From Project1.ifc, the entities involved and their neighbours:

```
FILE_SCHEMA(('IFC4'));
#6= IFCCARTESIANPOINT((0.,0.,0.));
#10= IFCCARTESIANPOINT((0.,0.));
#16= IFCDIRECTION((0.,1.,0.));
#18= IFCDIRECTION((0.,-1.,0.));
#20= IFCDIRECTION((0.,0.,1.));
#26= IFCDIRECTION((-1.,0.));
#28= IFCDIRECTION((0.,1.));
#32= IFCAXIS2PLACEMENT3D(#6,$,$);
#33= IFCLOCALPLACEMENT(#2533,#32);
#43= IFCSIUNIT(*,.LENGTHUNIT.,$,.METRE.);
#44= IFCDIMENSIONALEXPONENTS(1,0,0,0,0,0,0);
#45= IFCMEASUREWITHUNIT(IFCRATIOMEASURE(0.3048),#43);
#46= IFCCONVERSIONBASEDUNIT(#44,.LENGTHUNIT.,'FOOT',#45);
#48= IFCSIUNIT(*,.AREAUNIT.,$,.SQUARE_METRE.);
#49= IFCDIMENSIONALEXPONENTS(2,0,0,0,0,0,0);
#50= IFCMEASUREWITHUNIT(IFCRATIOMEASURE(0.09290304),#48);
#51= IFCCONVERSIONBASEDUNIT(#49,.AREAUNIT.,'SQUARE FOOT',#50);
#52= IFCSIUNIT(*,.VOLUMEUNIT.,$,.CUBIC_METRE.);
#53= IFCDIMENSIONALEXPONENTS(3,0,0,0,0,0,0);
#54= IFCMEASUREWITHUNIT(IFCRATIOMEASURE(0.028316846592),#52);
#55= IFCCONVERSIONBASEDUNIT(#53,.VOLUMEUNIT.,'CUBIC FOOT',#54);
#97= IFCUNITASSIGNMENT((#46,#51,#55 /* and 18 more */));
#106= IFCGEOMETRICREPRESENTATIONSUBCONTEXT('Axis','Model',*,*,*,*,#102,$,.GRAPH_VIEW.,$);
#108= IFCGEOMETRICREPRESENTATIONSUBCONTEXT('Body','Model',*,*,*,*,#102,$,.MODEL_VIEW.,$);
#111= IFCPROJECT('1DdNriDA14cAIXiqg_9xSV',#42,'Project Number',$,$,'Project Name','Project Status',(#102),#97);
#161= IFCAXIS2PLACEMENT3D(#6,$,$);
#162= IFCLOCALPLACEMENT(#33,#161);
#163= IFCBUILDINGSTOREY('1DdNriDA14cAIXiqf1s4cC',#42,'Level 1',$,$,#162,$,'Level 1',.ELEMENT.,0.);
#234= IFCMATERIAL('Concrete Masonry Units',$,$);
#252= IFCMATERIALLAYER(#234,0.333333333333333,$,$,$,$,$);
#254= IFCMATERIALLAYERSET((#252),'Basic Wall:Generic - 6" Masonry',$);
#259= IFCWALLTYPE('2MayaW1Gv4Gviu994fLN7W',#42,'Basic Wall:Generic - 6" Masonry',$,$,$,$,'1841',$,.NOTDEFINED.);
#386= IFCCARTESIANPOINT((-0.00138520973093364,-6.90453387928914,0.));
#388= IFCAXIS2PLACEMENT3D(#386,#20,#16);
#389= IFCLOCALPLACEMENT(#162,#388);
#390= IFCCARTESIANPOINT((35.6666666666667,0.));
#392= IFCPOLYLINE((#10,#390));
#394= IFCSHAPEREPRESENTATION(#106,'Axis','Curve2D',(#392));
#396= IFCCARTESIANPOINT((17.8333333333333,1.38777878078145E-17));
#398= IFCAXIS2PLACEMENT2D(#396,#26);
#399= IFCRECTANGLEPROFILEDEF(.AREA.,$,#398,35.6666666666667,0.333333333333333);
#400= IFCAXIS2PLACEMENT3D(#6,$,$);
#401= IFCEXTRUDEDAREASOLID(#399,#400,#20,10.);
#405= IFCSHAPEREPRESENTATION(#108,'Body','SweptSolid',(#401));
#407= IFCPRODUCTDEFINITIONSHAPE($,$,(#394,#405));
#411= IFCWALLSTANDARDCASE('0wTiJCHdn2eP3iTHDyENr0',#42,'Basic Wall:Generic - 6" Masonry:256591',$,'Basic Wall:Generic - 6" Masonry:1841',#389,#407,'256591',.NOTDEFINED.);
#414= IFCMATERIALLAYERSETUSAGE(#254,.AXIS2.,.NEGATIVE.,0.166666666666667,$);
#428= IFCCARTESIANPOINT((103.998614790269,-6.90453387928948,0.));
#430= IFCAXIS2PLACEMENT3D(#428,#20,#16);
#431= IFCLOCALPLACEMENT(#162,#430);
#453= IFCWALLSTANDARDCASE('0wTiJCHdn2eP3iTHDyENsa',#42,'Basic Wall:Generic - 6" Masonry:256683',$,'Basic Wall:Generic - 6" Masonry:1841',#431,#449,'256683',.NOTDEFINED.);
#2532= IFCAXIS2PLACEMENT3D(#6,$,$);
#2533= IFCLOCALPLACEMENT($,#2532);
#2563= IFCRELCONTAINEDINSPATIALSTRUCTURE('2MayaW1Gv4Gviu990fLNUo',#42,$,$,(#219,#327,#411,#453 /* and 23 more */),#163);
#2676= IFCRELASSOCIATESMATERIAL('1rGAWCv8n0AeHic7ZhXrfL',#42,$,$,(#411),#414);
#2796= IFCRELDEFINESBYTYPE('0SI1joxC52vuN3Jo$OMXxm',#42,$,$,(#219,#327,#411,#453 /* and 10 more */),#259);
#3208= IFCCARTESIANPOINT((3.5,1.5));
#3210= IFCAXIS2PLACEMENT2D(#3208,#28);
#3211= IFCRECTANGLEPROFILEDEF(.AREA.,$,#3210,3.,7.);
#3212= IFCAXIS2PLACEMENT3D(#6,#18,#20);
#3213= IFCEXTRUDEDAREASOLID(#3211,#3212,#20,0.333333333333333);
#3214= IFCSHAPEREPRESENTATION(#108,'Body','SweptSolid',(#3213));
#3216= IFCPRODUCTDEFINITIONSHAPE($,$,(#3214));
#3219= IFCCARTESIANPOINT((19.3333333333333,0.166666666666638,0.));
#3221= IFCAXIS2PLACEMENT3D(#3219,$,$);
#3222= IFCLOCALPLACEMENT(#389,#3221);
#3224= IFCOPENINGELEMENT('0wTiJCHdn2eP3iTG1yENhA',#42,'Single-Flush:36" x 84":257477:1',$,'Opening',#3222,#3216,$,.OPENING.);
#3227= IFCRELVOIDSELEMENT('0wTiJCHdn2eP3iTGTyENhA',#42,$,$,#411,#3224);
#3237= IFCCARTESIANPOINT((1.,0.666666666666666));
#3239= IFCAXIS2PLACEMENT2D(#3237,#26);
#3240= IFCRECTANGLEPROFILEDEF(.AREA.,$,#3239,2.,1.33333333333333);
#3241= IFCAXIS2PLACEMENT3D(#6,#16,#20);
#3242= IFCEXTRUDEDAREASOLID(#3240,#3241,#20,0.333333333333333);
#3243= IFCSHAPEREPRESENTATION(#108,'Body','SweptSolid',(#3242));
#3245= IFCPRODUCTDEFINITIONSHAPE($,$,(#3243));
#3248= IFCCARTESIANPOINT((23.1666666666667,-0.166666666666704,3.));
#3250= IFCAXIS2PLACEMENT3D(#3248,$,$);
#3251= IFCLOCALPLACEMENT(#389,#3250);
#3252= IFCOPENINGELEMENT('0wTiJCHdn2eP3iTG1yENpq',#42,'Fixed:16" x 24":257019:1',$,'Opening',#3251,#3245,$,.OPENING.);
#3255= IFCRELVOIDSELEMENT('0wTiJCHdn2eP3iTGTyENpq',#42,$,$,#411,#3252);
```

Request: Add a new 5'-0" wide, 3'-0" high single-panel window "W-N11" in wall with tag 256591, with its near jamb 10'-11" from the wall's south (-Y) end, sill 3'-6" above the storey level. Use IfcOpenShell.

```python
import numpy as np
import ifcopenshell
import ifcopenshell.api.feature
import ifcopenshell.api.geometry
import ifcopenshell.api.root
import ifcopenshell.api.spatial
import ifcopenshell.geom
import ifcopenshell.util.element
import ifcopenshell.util.placement
import ifcopenshell.util.representation
import ifcopenshell.util.shape
import ifcopenshell.util.unit

model = ifcopenshell.open("Project1.ifc")
unit_scale = ifcopenshell.util.unit.calculate_unit_scale(model)
settings = ifcopenshell.geom.settings()


def volume(element):
    """Net volume in cubic metres, openings subtracted."""
    shape = ifcopenshell.geom.create_shape(settings, element)
    return ifcopenshell.util.shape.get_volume(shape.geometry)


wall = model.by_id(411)
storey = ifcopenshell.util.element.get_container(wall, ifc_class="IfcBuildingStorey")
context = ifcopenshell.util.representation.get_context(model, "Model", "Body", "MODEL_VIEW")
before = volume(wall)

width, height, from_end, sill = 1.524, 0.9144, 3.3274, 1.0668  # metres

# The wall runs along its own X axis, and the end named is its -X end.
wall_shape = ifcopenshell.geom.create_shape(settings, wall)
x, y, z = ifcopenshell.util.shape.get_vertices(wall_shape.geometry).T
start = x.min() + from_end
face, thickness = float(y.min()), float(y.max() - y.min())
wall_matrix = ifcopenshell.util.placement.get_local_placement(wall.ObjectPlacement)
level = ifcopenshell.util.placement.get_local_placement(storey.ObjectPlacement)[2, 3]


def in_wall(x, y):
    """Placement at x, y metres in the wall's axes, at sill height."""
    matrix = wall_matrix.copy()
    matrix[:, 3] = wall_matrix @ np.array([x / unit_scale, y / unit_scale, 0.0, 1.0])
    matrix[2, 3] = level + sill / unit_scale
    return matrix


# Opening: a box that overshoots both wall faces by 50 mm.
opening = ifcopenshell.api.root.create_entity(model, ifc_class="IfcOpeningElement", predefined_type="OPENING")
box = ifcopenshell.api.geometry.add_wall_representation(
    model, context=context, length=width, height=height, thickness=thickness + 0.1
)
ifcopenshell.api.geometry.assign_representation(model, product=opening, representation=box)
ifcopenshell.api.geometry.edit_object_placement(model, product=opening, matrix=in_wall(start, face - 0.05), is_si=False)
ifcopenshell.api.feature.add_feature(model, feature=opening, element=wall)

window = ifcopenshell.api.root.create_entity(model, ifc_class="IfcWindow", name="W-N11", predefined_type="WINDOW")
window.OverallWidth, window.OverallHeight = width / unit_scale, height / unit_scale
window.PartitioningType = "SINGLE_PANEL"
body = ifcopenshell.api.geometry.add_window_representation(
    model,
    context=context,
    overall_width=window.OverallWidth,
    overall_height=window.OverallHeight,
    partition_type="SINGLE_PANEL",
)
ifcopenshell.api.geometry.assign_representation(model, product=window, representation=body)
ifcopenshell.api.spatial.assign_container(model, products=[window], relating_structure=storey)
ifcopenshell.api.feature.add_filling(model, opening=opening, element=window)

# Centre the window in the wall's thickness.
ifcopenshell.api.geometry.edit_object_placement(model, product=window, matrix=in_wall(start, face), is_si=False)
window_shape = ifcopenshell.geom.create_shape(settings, window)
depth = ifcopenshell.util.shape.get_vertices(window_shape.geometry)[:, 1]
offset = face + thickness / 2 - (depth.min() + depth.max()) / 2
ifcopenshell.api.geometry.edit_object_placement(model, product=window, matrix=in_wall(start, offset), is_si=False)

after = volume(wall)

print(f"wall volume {before:.3f} -> {after:.3f} m3")

model.write("Project1_rev.ifc")
```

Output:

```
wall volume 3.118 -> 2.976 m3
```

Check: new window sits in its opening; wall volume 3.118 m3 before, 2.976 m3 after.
